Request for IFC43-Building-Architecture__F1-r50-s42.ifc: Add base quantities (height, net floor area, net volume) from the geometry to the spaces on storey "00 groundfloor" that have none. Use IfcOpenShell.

First a look at what the model holds.

```python
import ifcopenshell
import ifcopenshell.util.element
import ifcopenshell.util.unit

model = ifcopenshell.open("IFC43-Building-Architecture__F1-r50-s42.ifc")
print(model.schema)
for unit_type in ("LENGTHUNIT", "AREAUNIT", "VOLUMEUNIT"):
    print(unit_type, ifcopenshell.util.unit.calculate_unit_scale(model, unit_type))
storey = next(s for s in model.by_type("IfcBuildingStorey") if s.Name == "00 groundfloor")
spaces = [e for e in ifcopenshell.util.element.get_decomposition(storey) if e.is_a("IfcSpace")]
for e in sorted(spaces, key=lambda e: e.id()):
    print(e.id(), e.is_a(), e.Name, list(ifcopenshell.util.element.get_psets(e, qtos_only=True)), sep=" | ")
```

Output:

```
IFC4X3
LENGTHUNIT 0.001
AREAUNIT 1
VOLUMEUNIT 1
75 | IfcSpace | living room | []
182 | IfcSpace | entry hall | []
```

```python
import ifcopenshell
import ifcopenshell.api.pset
import ifcopenshell.geom
import ifcopenshell.util.element
import ifcopenshell.util.shape
import ifcopenshell.util.unit

model = ifcopenshell.open("IFC43-Building-Architecture__F1-r50-s42.ifc")
unit_scale = ifcopenshell.util.unit.calculate_unit_scale(model)
area_scale = ifcopenshell.util.unit.calculate_unit_scale(model, "AREAUNIT")
volume_scale = ifcopenshell.util.unit.calculate_unit_scale(model, "VOLUMEUNIT")
settings = ifcopenshell.geom.settings()

storey = next(s for s in model.by_type("IfcBuildingStorey") if s.Name == "00 groundfloor")
spaces = [e for e in ifcopenshell.util.element.get_decomposition(storey) if e.is_a("IfcSpace")]

for e in sorted(spaces, key=lambda e: e.id()):
    if ifcopenshell.util.element.get_psets(e, qtos_only=True, should_inherit=False):
        continue
    # Geometry comes back in metres, in the element's own axes.
    shape = ifcopenshell.geom.create_shape(settings, e)
    values = {
        "Height": ifcopenshell.util.shape.get_z(shape.geometry) / unit_scale,
        "NetFloorArea": ifcopenshell.util.shape.get_footprint_area(shape.geometry) / area_scale,
        "NetVolume": ifcopenshell.util.shape.get_volume(shape.geometry) / volume_scale,
    }
    qto = ifcopenshell.api.pset.add_qto(model, product=e, name="Qto_SpaceBaseQuantities")
    ifcopenshell.api.pset.edit_qto(model, qto=qto, properties=values)
    print(e.id(), {k: round(v, 3) for k, v in values.items()})

model.write("IFC43-Building-Architecture__F1-r50-s42_rev.ifc")
```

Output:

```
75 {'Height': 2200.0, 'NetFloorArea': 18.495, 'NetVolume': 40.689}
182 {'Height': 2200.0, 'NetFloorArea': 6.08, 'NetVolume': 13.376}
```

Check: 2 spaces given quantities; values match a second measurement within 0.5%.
